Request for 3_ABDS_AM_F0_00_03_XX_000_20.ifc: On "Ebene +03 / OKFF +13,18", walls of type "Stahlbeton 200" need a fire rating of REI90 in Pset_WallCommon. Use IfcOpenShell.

First a look at what the model holds.

```python
import ifcopenshell
import ifcopenshell.util.element

model = ifcopenshell.open("3_ABDS_AM_F0_00_03_XX_000_20.ifc")
print(model.schema)
storey = next(s for s in model.by_type("IfcBuildingStorey") if s.Name == "Ebene +03 / OKFF +13,18")
walls = [e for e in ifcopenshell.util.element.get_decomposition(storey) if e.is_a("IfcWall")]
seen = {}
for e in walls:
    element_type = ifcopenshell.util.element.get_type(e)
    key = (element_type.Name if element_type != e and element_type else None, ifcopenshell.util.element.get_pset(e, "Pset_WallCommon", "FireRating"))
    seen[key] = seen.get(key, 0) + 1
for (name, value), count in sorted(seen.items(), key=str):
    print(count, "x", name, "|", value)
```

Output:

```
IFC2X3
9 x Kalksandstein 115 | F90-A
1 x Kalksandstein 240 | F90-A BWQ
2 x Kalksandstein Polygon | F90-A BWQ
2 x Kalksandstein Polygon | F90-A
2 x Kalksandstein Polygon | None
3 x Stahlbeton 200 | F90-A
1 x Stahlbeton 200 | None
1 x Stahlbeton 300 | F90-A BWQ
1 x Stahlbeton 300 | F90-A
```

```python
import ifcopenshell
import ifcopenshell.api.pset
import ifcopenshell.util.element

model = ifcopenshell.open("3_ABDS_AM_F0_00_03_XX_000_20.ifc")

storey = next(s for s in model.by_type("IfcBuildingStorey") if s.Name == "Ebene +03 / OKFF +13,18")
walls = [e for e in ifcopenshell.util.element.get_decomposition(storey) if e.is_a("IfcWall")]

count = 0
for e in walls:
    element_type = ifcopenshell.util.element.get_type(e)
    if element_type in (None, e) or element_type.Name != "Stahlbeton 200":
        continue
    # add_pset returns the element's existing set when there is one.
    pset = ifcopenshell.api.pset.add_pset(model, product=e, name="Pset_WallCommon")
    ifcopenshell.api.pset.edit_pset(model, pset=pset, properties={"FireRating": "REI90"})
    count += 1

print(count, "walls updated")

model.write("3_ABDS_AM_F0_00_03_XX_000_20-out.ifc")
```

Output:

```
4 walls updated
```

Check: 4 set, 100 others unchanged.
